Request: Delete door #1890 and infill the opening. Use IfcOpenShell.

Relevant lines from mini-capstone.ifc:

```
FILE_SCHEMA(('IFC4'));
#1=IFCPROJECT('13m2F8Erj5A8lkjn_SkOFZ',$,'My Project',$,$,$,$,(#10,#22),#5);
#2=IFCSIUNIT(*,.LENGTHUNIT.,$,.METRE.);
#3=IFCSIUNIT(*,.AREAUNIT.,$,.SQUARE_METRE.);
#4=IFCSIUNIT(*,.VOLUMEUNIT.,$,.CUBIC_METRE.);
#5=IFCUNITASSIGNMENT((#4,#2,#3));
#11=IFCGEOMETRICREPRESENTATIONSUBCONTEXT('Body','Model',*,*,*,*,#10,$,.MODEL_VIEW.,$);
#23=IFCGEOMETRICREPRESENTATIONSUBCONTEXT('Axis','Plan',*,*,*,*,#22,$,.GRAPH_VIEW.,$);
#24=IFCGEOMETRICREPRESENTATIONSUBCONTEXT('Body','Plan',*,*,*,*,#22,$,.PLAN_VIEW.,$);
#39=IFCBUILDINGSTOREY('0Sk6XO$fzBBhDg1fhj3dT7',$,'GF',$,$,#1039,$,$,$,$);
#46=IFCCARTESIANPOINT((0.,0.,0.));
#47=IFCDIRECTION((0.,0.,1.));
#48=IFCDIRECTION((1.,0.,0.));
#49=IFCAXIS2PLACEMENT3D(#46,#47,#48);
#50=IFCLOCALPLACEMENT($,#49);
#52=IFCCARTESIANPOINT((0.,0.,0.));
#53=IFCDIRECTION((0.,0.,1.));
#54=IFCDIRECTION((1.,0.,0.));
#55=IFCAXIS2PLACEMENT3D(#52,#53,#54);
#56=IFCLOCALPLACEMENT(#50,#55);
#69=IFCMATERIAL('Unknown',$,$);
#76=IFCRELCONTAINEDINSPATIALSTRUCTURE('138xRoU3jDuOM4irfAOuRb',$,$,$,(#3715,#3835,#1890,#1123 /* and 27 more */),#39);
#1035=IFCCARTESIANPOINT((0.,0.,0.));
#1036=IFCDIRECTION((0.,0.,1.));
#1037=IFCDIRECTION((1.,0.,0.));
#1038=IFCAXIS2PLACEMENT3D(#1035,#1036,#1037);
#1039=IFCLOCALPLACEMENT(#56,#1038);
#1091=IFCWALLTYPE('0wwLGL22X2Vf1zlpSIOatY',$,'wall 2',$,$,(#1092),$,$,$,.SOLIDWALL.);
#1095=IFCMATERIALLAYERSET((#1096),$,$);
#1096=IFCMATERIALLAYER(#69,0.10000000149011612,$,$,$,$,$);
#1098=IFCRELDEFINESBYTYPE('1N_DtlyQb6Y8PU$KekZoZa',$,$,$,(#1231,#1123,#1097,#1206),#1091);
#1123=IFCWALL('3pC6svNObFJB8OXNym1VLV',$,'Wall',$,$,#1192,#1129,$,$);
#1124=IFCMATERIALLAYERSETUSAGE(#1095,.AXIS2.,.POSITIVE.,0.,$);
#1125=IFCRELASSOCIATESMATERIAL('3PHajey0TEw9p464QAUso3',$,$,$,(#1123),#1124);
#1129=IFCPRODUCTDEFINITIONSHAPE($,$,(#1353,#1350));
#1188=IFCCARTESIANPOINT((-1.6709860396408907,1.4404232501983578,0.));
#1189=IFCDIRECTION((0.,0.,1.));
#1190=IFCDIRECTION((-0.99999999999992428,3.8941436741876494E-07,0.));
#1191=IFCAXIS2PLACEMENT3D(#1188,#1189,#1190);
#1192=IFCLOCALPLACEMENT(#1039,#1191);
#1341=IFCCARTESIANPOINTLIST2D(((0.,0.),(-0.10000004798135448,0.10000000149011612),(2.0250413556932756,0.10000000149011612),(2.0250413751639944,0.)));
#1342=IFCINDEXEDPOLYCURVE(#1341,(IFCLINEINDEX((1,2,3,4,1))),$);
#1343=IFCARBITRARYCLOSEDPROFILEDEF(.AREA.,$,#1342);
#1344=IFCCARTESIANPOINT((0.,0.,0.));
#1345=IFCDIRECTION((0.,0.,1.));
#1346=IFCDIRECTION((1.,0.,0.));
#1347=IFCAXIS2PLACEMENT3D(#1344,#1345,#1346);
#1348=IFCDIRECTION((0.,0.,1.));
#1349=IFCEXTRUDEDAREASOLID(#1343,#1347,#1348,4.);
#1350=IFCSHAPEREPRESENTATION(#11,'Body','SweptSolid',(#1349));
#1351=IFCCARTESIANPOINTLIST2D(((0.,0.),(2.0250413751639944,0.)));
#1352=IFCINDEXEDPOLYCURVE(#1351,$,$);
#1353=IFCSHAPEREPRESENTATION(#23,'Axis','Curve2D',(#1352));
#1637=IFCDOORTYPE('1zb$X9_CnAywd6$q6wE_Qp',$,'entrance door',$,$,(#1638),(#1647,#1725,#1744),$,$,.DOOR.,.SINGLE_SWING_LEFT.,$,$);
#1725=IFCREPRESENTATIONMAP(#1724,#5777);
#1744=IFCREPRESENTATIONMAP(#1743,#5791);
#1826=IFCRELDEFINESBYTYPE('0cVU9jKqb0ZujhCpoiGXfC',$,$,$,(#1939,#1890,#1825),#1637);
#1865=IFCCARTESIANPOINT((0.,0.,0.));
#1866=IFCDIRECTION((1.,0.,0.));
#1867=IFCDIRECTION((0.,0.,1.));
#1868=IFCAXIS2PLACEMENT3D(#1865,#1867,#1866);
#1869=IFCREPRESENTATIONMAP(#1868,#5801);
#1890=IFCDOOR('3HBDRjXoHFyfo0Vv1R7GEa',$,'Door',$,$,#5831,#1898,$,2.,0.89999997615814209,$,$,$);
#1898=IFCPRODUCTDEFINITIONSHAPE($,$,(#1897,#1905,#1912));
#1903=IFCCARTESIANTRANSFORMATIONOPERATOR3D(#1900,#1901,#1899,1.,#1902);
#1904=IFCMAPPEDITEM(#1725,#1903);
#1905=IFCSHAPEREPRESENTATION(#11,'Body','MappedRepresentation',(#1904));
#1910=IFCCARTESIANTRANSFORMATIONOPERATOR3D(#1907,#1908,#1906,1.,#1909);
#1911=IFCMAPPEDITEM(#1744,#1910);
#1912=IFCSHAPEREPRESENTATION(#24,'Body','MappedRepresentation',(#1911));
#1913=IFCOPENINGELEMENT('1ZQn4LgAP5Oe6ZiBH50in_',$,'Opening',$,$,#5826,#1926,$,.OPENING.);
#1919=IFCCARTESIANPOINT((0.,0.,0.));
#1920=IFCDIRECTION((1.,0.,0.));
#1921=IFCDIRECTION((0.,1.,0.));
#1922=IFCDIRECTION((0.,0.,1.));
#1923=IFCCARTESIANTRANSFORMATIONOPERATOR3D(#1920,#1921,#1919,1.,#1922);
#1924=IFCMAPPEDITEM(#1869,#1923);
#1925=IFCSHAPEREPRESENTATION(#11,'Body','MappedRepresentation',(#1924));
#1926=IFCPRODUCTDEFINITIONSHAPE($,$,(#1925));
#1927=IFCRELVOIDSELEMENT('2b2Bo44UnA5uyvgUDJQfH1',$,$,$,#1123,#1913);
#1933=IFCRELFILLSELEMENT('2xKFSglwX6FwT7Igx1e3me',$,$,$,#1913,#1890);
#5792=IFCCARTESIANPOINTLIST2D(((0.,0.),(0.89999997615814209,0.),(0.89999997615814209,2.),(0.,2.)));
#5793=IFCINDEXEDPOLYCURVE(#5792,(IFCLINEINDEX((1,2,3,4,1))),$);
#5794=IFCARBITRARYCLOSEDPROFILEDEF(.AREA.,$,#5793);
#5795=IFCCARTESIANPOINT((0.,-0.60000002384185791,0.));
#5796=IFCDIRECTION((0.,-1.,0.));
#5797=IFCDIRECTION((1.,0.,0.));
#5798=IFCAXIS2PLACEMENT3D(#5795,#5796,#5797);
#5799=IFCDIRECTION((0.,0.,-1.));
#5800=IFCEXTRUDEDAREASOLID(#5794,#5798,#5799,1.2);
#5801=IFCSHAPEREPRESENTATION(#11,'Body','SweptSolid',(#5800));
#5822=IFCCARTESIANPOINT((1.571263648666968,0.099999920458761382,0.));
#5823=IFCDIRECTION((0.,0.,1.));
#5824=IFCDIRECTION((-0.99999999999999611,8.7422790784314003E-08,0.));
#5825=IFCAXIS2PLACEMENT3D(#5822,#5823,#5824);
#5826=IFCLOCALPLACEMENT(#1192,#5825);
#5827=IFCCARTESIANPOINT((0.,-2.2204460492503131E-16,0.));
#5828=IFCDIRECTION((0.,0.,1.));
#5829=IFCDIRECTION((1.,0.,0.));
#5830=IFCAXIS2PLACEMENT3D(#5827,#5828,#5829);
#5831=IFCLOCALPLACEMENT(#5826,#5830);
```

```python
import ifcopenshell
import ifcopenshell.api.feature
import ifcopenshell.api.root
import ifcopenshell.geom
import ifcopenshell.util.shape

model = ifcopenshell.open("mini-capstone.ifc")
settings = ifcopenshell.geom.settings()


def volume(element):
    """Net volume in cubic metres, openings subtracted."""
    shape = ifcopenshell.geom.create_shape(settings, element)
    return ifcopenshell.util.shape.get_volume(shape.geometry)


door = model.by_guid("3HBDRjXoHFyfo0Vv1R7GEa")
opening = door.FillsVoids[0].RelatingOpeningElement
wall = opening.VoidsElements[0].RelatingBuildingElement
before = volume(wall)

ifcopenshell.api.root.remove_product(model, product=door)
ifcopenshell.api.feature.remove_feature(model, feature=opening)

after = volume(wall)

print(f"wall volume {before:.3f} -> {after:.3f} m3")

model.write("mini-capstone_edited.ifc")
```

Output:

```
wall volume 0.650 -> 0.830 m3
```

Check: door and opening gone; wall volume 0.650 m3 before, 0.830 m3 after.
